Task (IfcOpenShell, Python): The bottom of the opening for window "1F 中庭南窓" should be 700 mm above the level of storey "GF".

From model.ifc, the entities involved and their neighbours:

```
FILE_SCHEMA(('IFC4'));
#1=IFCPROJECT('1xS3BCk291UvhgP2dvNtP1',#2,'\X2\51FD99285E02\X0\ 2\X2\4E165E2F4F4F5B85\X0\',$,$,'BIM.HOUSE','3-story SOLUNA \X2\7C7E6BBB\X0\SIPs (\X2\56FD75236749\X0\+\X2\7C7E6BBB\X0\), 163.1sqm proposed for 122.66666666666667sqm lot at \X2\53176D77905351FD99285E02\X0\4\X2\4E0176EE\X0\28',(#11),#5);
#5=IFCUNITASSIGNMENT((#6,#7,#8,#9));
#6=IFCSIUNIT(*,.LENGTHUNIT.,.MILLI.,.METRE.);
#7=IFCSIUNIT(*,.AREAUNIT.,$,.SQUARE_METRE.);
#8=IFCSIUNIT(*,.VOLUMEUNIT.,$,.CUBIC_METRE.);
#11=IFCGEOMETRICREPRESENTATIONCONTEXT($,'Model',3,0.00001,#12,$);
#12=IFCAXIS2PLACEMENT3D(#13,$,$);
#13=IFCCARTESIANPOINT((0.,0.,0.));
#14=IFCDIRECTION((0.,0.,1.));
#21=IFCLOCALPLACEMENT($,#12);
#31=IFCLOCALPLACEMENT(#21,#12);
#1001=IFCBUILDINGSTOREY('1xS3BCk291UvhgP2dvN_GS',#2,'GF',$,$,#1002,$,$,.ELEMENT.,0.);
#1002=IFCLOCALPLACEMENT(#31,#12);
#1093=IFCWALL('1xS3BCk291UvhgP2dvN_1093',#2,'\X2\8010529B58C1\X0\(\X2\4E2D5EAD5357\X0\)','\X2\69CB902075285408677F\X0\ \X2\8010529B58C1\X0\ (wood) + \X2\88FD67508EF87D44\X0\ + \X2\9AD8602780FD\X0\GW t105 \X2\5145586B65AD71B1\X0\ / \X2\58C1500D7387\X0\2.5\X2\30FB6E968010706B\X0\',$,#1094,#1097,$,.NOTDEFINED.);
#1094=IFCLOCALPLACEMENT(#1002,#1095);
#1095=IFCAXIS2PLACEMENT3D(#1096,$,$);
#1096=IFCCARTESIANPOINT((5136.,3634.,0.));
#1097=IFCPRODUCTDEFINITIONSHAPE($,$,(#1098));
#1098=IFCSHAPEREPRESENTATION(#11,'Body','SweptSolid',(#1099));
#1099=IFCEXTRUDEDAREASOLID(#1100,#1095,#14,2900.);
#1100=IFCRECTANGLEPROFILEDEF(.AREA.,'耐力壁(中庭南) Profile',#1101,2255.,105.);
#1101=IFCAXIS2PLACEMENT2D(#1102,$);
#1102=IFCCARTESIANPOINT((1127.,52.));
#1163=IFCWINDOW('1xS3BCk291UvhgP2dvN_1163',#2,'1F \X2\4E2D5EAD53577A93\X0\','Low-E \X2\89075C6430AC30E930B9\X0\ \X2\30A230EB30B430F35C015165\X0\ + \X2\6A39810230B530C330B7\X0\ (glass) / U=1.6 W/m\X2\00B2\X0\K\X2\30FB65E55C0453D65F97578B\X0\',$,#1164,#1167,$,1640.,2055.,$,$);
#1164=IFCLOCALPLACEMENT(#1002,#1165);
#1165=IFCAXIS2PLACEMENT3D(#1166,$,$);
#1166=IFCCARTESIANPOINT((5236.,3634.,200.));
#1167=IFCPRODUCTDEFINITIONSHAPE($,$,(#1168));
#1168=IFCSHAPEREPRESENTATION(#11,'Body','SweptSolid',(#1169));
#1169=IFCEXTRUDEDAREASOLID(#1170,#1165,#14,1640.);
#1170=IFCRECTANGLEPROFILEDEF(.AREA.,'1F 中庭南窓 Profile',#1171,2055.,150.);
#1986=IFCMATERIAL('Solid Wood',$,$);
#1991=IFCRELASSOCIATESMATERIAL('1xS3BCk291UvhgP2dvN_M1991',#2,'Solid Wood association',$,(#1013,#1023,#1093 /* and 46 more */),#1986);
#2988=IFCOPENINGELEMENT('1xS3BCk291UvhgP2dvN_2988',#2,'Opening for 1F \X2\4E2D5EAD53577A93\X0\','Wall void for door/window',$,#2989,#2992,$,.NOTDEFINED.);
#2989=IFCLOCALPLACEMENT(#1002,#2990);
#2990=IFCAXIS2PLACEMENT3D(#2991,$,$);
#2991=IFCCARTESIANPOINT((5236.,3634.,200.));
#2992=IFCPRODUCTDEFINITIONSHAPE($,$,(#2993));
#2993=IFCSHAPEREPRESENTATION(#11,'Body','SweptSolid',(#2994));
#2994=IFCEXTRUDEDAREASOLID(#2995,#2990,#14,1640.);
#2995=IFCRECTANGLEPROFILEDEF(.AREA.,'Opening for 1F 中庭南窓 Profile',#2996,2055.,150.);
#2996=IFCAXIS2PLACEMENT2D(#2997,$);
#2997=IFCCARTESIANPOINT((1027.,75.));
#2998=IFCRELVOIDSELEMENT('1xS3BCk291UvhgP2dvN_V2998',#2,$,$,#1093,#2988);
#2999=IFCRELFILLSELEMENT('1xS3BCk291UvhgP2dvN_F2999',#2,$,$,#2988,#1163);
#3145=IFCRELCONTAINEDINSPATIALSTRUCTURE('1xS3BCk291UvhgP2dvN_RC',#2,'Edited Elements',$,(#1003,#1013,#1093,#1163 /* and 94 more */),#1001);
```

```python
import numpy as np
import ifcopenshell
import ifcopenshell.api.geometry
import ifcopenshell.geom
import ifcopenshell.util.element
import ifcopenshell.util.placement
import ifcopenshell.util.shape
import ifcopenshell.util.unit

model = ifcopenshell.open("model.ifc")
unit_scale = ifcopenshell.util.unit.calculate_unit_scale(model)

window = model.by_id(1163)
opening = window.FillsVoids[0].RelatingOpeningElement
storey = ifcopenshell.util.element.get_container(window, ifc_class="IfcBuildingStorey")
level = ifcopenshell.util.placement.get_local_placement(storey.ObjectPlacement)[2, 3]

# The opening's origin need not be at the sill, so measure its lowest point.
shape = ifcopenshell.geom.create_shape(ifcopenshell.geom.settings(), opening)
bottom = ifcopenshell.util.shape.get_shape_bottom_elevation(shape, shape.geometry) / unit_scale
dz = level + 700.0 - bottom

shift = np.array([0.0, 0.0, dz])
# The window is not placed relative to its opening, so move both.
for product in (opening, window):
    matrix = ifcopenshell.util.placement.get_local_placement(product.ObjectPlacement)
    matrix[:3, 3] += shift
    ifcopenshell.api.geometry.edit_object_placement(model, product=product, matrix=matrix, is_si=False)

print(f"moved by {dz * unit_scale:+.3f} m")

model.write("model_edited.ifc")
```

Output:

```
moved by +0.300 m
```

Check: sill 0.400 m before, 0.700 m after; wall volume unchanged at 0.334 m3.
